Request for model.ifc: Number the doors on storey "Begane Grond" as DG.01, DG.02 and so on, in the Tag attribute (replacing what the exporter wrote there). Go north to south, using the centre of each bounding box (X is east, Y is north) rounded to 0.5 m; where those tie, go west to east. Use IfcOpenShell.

First a look at what the model holds.

```python
import ifcopenshell
import ifcopenshell.util.element
import ifcopenshell.util.placement

model = ifcopenshell.open("model.ifc")
print(model.schema)
storey = next(s for s in model.by_type("IfcBuildingStorey") if s.Name == "Begane Grond")
doors = [e for e in ifcopenshell.util.element.get_decomposition(storey) if e.is_a("IfcDoor")]
for e in sorted(doors, key=lambda e: e.id()):
    origin = ifcopenshell.util.placement.get_local_placement(e.ObjectPlacement)[:3, 3]
    print(e.id(), e.Tag, e.Name, origin.round(2) + 0.0, sep=" | ")
```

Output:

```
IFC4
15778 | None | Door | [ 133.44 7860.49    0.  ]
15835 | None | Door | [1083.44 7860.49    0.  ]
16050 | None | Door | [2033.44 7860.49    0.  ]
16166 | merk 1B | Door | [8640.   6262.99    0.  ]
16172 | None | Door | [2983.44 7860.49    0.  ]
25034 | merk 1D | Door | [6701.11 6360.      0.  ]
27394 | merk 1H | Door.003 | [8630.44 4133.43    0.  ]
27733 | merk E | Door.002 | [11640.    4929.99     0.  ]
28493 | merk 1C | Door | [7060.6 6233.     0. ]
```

```python
import ifcopenshell
import ifcopenshell.geom
import ifcopenshell.util.element
import ifcopenshell.util.shape

model = ifcopenshell.open("model.ifc")
settings = ifcopenshell.geom.settings()
settings.set("use-world-coords", True)


def centre(element):
    shape = ifcopenshell.geom.create_shape(settings, element)
    return ifcopenshell.util.shape.get_bbox_centroid(shape.geometry)


storey = next(s for s in model.by_type("IfcBuildingStorey") if s.Name == "Begane Grond")
doors = [e for e in ifcopenshell.util.element.get_decomposition(storey) if e.is_a("IfcDoor")]

# Insertion points can sit at a corner or the storey origin, so sort by the geometry (in metres).
centres = {e: centre(e) for e in doors}
doors.sort(key=lambda e: (-round(centres[e][1] / 0.5), centres[e][0]))

for i, e in enumerate(doors, start=1):
    number = f"DG.{i:02d}"
    e.Tag = number
    print(e.id(), number)

model.write("model_rev.ifc")
```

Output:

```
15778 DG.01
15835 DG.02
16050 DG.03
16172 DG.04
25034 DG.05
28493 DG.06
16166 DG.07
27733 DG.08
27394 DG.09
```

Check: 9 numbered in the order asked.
